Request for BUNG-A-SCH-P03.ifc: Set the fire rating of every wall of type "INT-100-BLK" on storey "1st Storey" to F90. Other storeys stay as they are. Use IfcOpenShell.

First a look at what the model holds.

```python
import ifcopenshell
import ifcopenshell.util.element

model = ifcopenshell.open("BUNG-A-SCH-P03.ifc")
print(model.schema)
storey = next(s for s in model.by_type("IfcBuildingStorey") if s.Name == "1st Storey")
walls = [e for e in ifcopenshell.util.element.get_decomposition(storey) if e.is_a("IfcWall")]
seen = {}
for e in walls:
    element_type = ifcopenshell.util.element.get_type(e)
    key = (element_type.Name if element_type != e and element_type else None, ifcopenshell.util.element.get_pset(e, "Pset_WallCommon", "FireRating"))
    seen[key] = seen.get(key, 0) + 1
for (name, value), count in sorted(seen.items(), key=str):
    print(count, "x", name, "|", value)
```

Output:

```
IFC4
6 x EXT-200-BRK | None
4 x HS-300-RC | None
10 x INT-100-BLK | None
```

```python
import ifcopenshell
import ifcopenshell.api.pset
import ifcopenshell.util.element

model = ifcopenshell.open("BUNG-A-SCH-P03.ifc")

storey = next(s for s in model.by_type("IfcBuildingStorey") if s.Name == "1st Storey")
walls = [e for e in ifcopenshell.util.element.get_decomposition(storey) if e.is_a("IfcWall")]

count = 0
for e in walls:
    element_type = ifcopenshell.util.element.get_type(e)
    if element_type in (None, e) or element_type.Name != "INT-100-BLK":
        continue
    # add_pset returns the element's existing set when there is one.
    pset = ifcopenshell.api.pset.add_pset(model, product=e, name="Pset_WallCommon")
    ifcopenshell.api.pset.edit_pset(model, pset=pset, properties={"FireRating": "F90"})
    count += 1

print(count, "walls updated")

model.write("BUNG-A-SCH-P03_updated.ifc")
```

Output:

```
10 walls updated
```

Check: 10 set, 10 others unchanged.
